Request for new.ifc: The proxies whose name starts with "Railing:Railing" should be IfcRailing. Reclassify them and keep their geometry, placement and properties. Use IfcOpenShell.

First a look at what the model holds.

```python
import re

import ifcopenshell

model = ifcopenshell.open("new.ifc")
print(model.schema)
seen = {}
for e in model.by_type("IfcBuildingElementProxy"):
    name = re.sub(r":\d+(:\d+)?$", "", e.Name or "")  # drop the element id that some exporters append
    seen[name] = seen.get(name, 0) + 1
for name, count in sorted(seen.items()):
    print(count, "x", name)
```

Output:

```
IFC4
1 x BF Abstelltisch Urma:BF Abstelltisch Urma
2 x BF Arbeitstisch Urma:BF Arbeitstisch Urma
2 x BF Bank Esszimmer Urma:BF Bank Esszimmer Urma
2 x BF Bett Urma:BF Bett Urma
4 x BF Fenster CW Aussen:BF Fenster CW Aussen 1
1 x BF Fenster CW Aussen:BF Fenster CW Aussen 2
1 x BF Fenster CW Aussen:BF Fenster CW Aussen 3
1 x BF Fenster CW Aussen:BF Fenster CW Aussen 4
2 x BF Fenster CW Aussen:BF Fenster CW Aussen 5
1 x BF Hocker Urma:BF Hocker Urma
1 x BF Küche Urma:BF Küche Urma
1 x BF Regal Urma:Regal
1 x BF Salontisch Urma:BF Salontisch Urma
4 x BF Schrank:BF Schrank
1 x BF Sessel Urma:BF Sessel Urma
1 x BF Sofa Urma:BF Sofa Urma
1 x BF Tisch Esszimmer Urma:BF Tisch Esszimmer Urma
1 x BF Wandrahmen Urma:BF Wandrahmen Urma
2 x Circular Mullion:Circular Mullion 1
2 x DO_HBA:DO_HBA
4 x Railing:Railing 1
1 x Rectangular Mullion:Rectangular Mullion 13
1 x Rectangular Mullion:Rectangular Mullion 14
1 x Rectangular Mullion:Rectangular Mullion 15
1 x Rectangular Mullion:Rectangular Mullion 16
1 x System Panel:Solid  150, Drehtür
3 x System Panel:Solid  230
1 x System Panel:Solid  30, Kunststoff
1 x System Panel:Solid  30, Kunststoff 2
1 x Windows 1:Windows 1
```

```python
import ifcopenshell
import ifcopenshell.api.root

model = ifcopenshell.open("new.ifc")

proxies = [e.id() for e in model.by_type("IfcBuildingElementProxy") if (e.Name or "").startswith("Railing:Railing")]
for step_id in proxies:
    proxy = model.by_id(step_id)
    ifcopenshell.api.root.reassign_class(model, product=proxy, ifc_class="IfcRailing")

print(sum(model.by_id(i).is_a("IfcRailing") for i in proxies), "reclassified")

model.write("new_updated.ifc")
```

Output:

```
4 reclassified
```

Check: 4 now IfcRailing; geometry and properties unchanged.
